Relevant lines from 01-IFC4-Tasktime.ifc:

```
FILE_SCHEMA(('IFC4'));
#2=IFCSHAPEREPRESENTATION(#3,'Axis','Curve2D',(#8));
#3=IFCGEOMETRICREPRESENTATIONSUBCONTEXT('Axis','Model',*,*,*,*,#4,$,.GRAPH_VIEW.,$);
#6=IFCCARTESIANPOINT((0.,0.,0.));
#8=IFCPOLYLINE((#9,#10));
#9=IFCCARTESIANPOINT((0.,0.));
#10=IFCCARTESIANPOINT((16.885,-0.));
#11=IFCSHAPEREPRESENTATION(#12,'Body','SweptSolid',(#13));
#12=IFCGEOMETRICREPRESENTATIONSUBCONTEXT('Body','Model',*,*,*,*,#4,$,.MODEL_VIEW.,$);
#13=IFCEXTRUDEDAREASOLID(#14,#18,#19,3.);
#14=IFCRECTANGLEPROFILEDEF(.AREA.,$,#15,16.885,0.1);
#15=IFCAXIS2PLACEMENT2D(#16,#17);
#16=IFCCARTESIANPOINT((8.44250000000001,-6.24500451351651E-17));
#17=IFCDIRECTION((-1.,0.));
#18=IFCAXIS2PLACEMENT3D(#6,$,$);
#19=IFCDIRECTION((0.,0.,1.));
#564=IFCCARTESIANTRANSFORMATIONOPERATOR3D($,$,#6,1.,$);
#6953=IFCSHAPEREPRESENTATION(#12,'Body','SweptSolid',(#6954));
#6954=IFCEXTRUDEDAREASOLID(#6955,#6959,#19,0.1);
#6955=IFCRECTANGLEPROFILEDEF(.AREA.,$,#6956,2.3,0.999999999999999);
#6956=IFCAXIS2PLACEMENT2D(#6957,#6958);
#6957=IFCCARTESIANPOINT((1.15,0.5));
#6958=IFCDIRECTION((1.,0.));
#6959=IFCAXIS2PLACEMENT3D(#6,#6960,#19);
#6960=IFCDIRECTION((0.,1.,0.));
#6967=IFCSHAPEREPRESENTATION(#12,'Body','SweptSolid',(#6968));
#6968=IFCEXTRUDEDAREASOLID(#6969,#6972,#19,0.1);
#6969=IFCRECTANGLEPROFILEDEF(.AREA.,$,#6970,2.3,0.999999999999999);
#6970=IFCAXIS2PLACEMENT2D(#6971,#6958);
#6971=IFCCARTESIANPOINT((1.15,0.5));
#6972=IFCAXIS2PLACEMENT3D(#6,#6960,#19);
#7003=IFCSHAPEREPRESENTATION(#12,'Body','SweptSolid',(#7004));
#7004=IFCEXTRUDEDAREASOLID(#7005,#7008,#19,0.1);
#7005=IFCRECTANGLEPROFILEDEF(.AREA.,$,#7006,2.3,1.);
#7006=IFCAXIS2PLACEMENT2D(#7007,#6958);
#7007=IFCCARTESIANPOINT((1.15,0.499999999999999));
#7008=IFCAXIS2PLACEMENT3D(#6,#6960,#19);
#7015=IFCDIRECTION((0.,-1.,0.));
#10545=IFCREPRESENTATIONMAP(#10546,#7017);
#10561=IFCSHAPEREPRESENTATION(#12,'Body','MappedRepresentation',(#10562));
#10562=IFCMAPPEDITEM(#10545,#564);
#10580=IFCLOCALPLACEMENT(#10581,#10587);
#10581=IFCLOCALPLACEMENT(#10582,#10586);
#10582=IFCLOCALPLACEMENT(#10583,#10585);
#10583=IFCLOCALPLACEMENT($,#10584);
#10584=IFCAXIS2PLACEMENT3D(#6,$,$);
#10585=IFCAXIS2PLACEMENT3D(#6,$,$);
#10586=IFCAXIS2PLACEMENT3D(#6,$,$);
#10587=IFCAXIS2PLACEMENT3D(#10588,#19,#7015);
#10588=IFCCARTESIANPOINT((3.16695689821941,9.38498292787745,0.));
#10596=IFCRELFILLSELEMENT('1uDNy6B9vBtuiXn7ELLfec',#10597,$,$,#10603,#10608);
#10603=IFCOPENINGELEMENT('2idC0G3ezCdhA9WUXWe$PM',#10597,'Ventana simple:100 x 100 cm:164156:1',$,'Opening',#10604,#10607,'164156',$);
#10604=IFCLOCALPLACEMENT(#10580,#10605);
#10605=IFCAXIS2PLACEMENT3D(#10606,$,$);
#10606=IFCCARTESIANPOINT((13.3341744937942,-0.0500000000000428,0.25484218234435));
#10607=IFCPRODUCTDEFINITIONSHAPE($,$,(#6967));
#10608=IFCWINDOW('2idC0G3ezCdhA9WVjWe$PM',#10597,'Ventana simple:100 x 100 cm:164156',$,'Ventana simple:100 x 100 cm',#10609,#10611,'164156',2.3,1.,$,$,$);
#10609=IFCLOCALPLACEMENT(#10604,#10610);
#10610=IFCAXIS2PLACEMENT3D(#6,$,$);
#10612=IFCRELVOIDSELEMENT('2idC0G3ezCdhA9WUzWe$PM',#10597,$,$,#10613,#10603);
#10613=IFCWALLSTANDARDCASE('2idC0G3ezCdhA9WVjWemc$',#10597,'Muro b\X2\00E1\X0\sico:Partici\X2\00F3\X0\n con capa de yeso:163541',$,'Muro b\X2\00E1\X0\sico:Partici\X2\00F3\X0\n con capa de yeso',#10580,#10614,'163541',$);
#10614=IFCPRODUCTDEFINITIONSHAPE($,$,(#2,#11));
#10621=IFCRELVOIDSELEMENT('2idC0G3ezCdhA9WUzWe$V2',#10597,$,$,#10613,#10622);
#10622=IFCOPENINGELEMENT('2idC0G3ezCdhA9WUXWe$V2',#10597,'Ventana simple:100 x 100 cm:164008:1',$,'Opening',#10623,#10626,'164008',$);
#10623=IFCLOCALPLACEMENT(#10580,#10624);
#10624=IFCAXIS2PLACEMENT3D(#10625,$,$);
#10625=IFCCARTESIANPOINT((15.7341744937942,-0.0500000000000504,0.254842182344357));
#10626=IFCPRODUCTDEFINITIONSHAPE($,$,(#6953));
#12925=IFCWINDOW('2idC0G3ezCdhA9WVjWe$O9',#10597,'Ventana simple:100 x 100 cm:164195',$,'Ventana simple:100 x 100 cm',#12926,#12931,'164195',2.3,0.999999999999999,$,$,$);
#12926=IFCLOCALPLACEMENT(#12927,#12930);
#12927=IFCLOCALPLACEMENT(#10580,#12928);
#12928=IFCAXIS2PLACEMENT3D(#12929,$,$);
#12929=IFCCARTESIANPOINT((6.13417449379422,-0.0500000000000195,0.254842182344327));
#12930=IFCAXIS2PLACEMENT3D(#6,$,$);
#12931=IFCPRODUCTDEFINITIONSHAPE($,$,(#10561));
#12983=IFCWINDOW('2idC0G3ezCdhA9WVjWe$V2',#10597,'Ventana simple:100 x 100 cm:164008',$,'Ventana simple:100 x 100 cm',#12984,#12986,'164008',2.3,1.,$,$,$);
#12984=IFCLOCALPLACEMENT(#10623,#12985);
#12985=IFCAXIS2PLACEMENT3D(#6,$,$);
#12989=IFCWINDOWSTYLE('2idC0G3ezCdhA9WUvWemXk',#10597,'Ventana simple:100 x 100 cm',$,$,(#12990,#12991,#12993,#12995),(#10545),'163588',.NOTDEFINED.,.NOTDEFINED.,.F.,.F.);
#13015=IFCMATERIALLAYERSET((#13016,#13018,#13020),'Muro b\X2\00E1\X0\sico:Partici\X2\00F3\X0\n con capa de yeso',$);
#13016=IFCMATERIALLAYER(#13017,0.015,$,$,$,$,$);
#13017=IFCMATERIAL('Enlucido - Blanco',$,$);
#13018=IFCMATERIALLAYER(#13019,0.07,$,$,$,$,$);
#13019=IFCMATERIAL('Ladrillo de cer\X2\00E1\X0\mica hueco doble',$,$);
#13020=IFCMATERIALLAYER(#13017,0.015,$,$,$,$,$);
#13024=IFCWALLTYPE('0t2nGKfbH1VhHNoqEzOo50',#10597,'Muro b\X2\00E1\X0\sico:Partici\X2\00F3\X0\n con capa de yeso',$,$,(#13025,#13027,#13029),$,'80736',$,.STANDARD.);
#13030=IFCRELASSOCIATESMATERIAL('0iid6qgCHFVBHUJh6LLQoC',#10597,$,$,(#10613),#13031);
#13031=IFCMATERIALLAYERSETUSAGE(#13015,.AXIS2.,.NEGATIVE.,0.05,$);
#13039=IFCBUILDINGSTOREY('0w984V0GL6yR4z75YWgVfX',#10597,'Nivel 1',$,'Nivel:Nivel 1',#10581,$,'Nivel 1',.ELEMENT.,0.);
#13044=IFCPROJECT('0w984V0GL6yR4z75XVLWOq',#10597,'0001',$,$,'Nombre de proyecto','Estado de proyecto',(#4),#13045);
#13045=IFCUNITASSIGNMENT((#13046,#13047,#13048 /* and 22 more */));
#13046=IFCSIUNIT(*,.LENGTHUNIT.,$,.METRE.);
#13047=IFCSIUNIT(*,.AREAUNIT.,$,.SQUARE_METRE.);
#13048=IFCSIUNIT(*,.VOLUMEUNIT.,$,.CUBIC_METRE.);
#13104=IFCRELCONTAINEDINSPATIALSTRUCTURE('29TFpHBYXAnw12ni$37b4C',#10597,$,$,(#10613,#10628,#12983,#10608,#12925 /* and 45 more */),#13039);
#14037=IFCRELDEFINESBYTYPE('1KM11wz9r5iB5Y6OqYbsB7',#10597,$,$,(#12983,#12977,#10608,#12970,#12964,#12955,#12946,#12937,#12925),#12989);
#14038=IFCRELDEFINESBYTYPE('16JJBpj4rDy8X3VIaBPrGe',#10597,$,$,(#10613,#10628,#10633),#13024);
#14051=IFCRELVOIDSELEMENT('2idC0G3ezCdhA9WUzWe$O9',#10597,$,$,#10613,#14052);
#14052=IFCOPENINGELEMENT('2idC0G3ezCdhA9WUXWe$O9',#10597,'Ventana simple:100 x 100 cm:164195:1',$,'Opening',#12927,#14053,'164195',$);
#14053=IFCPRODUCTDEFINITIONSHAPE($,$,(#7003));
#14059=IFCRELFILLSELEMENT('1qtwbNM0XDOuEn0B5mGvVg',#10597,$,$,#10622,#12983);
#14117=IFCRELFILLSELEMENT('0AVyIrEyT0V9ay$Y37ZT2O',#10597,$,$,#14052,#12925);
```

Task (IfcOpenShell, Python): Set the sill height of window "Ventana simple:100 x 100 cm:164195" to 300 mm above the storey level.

```python
import numpy as np
import ifcopenshell
import ifcopenshell.api.geometry
import ifcopenshell.geom
import ifcopenshell.util.element
import ifcopenshell.util.placement
import ifcopenshell.util.shape
import ifcopenshell.util.unit

model = ifcopenshell.open("01-IFC4-Tasktime.ifc")
unit_scale = ifcopenshell.util.unit.calculate_unit_scale(model)

window = model.by_guid("2idC0G3ezCdhA9WVjWe$O9")
opening = window.FillsVoids[0].RelatingOpeningElement
storey = ifcopenshell.util.element.get_container(window, ifc_class="IfcBuildingStorey")
level = ifcopenshell.util.placement.get_local_placement(storey.ObjectPlacement)[2, 3]

# The opening's origin need not be at the sill, so measure its lowest point.
shape = ifcopenshell.geom.create_shape(ifcopenshell.geom.settings(), opening)
bottom = ifcopenshell.util.shape.get_shape_bottom_elevation(shape, shape.geometry) / unit_scale
dz = level + 0.3 - bottom

shift = np.array([0.0, 0.0, dz])
# The window is placed relative to its opening, so it follows when the opening moves.
matrix = ifcopenshell.util.placement.get_local_placement(opening.ObjectPlacement)
matrix[:3, 3] += shift
ifcopenshell.api.geometry.edit_object_placement(
    model, product=opening, matrix=matrix, is_si=False, should_transform_children=True
)

print(f"moved by {dz * unit_scale:+.3f} m")

model.write("01-IFC4-Tasktime_v2.ifc")
```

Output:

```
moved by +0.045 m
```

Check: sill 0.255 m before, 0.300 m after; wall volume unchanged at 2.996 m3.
